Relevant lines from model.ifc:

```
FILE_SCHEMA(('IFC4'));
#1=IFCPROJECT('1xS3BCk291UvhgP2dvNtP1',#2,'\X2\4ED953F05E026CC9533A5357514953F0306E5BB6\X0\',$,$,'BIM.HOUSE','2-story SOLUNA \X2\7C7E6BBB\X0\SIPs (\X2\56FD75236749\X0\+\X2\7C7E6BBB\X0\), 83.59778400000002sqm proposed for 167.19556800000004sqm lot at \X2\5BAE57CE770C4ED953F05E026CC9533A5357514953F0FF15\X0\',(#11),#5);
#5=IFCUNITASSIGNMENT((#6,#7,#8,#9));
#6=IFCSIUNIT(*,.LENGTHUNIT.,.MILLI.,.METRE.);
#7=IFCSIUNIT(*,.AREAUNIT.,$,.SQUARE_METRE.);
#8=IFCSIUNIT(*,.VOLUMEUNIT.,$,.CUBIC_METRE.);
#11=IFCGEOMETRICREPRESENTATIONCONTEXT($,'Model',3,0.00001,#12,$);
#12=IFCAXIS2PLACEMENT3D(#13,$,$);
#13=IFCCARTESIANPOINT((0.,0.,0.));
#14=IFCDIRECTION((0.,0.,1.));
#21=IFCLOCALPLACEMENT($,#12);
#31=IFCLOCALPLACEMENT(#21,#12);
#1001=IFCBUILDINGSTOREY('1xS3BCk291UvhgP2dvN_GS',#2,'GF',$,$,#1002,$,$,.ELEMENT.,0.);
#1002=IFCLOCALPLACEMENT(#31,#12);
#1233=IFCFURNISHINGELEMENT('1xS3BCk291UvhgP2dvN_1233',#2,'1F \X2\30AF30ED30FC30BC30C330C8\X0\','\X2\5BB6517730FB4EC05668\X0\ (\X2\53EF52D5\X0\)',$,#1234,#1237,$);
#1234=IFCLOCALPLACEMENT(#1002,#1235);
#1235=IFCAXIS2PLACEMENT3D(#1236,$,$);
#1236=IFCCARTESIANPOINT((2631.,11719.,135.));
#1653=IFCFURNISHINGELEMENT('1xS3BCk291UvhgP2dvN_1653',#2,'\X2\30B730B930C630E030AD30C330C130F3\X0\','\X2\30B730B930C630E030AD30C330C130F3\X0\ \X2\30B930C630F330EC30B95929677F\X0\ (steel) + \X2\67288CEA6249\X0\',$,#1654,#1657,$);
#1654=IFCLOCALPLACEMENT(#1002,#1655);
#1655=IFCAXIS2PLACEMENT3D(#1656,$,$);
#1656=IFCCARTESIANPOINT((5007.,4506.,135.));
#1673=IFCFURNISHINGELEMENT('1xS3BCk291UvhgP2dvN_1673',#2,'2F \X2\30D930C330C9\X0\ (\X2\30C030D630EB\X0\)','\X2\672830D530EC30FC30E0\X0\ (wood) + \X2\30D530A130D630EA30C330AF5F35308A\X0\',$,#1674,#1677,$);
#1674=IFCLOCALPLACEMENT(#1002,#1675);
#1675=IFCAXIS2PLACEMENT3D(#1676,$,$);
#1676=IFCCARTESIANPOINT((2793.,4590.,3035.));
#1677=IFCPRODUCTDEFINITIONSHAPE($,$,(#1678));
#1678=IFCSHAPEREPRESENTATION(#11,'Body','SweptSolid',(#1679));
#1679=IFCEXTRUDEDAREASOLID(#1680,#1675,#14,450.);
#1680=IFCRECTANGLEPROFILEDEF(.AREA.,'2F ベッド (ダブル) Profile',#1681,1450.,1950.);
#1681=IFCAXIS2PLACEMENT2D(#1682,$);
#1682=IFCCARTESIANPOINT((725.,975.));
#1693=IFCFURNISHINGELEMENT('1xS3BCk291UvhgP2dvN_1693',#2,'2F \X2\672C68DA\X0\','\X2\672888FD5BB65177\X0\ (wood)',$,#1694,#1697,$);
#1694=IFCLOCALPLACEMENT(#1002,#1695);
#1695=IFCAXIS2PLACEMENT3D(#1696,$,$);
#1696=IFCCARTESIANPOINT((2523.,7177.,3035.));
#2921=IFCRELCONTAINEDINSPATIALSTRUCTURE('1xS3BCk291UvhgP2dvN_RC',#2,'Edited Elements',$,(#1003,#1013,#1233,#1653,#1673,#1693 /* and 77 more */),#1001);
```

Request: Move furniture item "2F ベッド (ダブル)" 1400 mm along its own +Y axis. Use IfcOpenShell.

```python
import ifcopenshell
import ifcopenshell.api.geometry
import ifcopenshell.util.placement
import ifcopenshell.util.unit

model = ifcopenshell.open("model.ifc")
unit_scale = ifcopenshell.util.unit.calculate_unit_scale(model)

item = model.by_guid("1xS3BCk291UvhgP2dvN_1673")
matrix = ifcopenshell.util.placement.get_local_placement(item.ObjectPlacement)
matrix[:3, 3] += matrix[:3, 1] * 1.4 / unit_scale
ifcopenshell.api.geometry.edit_object_placement(model, product=item, matrix=matrix, is_si=False)

print(ifcopenshell.util.placement.get_local_placement(item.ObjectPlacement).round(3) + 0.0)

model.write("model_v2.ifc")
```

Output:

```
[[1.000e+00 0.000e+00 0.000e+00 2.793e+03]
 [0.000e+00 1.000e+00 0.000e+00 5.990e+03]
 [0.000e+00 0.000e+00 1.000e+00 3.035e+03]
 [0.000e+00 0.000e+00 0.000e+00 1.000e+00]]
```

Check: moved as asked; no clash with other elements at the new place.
